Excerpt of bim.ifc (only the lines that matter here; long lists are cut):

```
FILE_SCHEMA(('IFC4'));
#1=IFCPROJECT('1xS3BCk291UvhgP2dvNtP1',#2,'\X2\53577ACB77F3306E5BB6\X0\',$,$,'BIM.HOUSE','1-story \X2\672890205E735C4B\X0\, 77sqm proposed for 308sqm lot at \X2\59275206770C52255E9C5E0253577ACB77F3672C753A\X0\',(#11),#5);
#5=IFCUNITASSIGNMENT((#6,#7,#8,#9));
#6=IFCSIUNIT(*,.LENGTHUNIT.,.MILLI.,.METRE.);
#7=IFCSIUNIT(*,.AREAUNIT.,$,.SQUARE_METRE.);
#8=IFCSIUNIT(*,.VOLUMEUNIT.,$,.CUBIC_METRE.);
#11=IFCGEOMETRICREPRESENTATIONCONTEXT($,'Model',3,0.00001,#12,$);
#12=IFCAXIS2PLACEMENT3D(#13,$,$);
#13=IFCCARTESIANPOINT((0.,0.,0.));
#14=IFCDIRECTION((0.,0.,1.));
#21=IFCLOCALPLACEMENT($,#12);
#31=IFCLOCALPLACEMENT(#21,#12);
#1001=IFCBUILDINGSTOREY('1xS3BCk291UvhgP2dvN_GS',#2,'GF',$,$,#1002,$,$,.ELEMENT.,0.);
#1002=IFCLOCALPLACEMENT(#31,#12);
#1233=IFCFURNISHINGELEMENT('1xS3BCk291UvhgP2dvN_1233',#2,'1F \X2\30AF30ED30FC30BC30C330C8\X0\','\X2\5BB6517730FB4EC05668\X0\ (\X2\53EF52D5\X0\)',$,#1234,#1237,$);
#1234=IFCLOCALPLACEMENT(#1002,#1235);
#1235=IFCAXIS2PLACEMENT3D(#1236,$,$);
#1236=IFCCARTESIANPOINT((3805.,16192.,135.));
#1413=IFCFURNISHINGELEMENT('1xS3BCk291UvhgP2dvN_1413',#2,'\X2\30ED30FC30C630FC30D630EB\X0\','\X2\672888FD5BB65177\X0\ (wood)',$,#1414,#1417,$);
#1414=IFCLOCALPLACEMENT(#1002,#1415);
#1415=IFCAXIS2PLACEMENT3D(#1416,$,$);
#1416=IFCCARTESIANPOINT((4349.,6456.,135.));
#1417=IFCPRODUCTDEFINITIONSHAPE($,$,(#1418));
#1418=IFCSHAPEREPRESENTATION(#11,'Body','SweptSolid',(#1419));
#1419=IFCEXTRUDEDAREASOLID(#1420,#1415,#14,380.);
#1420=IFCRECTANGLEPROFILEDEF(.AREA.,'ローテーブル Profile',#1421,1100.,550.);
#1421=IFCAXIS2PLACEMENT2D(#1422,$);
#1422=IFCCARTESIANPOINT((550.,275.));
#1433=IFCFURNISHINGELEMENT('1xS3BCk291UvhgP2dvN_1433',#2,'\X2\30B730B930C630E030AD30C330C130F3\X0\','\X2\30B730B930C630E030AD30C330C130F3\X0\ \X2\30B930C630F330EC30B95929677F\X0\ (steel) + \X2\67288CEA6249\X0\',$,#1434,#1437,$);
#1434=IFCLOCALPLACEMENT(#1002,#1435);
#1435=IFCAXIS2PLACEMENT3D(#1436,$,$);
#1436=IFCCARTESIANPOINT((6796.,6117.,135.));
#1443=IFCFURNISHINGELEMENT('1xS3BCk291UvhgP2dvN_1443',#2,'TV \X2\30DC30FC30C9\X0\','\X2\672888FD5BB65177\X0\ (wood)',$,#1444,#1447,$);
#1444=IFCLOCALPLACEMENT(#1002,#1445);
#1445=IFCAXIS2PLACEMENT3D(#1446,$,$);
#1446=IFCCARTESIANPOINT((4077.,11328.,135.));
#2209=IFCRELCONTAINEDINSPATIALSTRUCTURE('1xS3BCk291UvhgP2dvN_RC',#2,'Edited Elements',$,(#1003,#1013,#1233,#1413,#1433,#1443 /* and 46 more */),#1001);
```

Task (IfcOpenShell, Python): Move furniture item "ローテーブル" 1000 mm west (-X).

```python
import ifcopenshell
import ifcopenshell.api.geometry
import ifcopenshell.util.placement
import ifcopenshell.util.unit

model = ifcopenshell.open("bim.ifc")
unit_scale = ifcopenshell.util.unit.calculate_unit_scale(model)

item = model.by_id(1413)
matrix = ifcopenshell.util.placement.get_local_placement(item.ObjectPlacement)
matrix[0, 3] -= 1 / unit_scale
ifcopenshell.api.geometry.edit_object_placement(model, product=item, matrix=matrix, is_si=False)

print(ifcopenshell.util.placement.get_local_placement(item.ObjectPlacement).round(3) + 0.0)

model.write("bim_edited.ifc")
```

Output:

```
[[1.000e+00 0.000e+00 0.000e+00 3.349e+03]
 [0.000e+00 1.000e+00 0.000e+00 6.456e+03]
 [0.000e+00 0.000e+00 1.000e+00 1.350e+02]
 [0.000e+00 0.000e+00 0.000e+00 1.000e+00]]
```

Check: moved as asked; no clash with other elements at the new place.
